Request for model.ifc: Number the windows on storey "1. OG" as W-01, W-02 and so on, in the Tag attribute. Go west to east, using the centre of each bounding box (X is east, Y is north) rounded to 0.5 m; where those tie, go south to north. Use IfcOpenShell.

First a look at what the model holds.

```python
import ifcopenshell
import ifcopenshell.util.element
import ifcopenshell.util.placement

model = ifcopenshell.open("model.ifc")
print(model.schema)
storey = next(s for s in model.by_type("IfcBuildingStorey") if s.Name == "1. OG")
windows = [e for e in ifcopenshell.util.element.get_decomposition(storey) if e.is_a("IfcWindow")]
for e in sorted(windows, key=lambda e: e.id()):
    origin = ifcopenshell.util.placement.get_local_placement(e.ObjectPlacement)[:3, 3]
    print(e.id(), e.Tag, e.Name, origin.round(2) + 0.0, sep=" | ")
```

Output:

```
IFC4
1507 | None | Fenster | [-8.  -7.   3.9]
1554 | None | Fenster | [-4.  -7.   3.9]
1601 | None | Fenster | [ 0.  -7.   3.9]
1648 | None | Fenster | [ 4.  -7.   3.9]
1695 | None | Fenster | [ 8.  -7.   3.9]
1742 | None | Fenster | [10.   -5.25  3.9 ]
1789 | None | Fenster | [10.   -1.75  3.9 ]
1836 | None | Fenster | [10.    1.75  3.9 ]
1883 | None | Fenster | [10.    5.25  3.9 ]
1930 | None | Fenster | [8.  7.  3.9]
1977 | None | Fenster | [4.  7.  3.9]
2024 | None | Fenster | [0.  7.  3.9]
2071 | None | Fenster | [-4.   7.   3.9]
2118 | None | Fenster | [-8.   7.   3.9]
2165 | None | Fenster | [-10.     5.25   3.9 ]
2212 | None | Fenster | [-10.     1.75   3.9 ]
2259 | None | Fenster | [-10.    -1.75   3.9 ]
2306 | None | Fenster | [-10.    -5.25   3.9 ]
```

```python
import ifcopenshell
import ifcopenshell.geom
import ifcopenshell.util.element
import ifcopenshell.util.shape

model = ifcopenshell.open("model.ifc")
settings = ifcopenshell.geom.settings()
settings.set("use-world-coords", True)


def centre(element):
    shape = ifcopenshell.geom.create_shape(settings, element)
    return ifcopenshell.util.shape.get_bbox_centroid(shape.geometry)


storey = next(s for s in model.by_type("IfcBuildingStorey") if s.Name == "1. OG")
windows = [e for e in ifcopenshell.util.element.get_decomposition(storey) if e.is_a("IfcWindow")]

# Insertion points can sit at a corner or the storey origin, so sort by the geometry (in metres).
centres = {e: centre(e) for e in windows}
windows.sort(key=lambda e: (round(centres[e][0] / 0.5), centres[e][1]))

for i, e in enumerate(windows, start=1):
    number = f"W-{i:02d}"
    e.Tag = number
    print(e.id(), number)

model.write("model_rev.ifc")
```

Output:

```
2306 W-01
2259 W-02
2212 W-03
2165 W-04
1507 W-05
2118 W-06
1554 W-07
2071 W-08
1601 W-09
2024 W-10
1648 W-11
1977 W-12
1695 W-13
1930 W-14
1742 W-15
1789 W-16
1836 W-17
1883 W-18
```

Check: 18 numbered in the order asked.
